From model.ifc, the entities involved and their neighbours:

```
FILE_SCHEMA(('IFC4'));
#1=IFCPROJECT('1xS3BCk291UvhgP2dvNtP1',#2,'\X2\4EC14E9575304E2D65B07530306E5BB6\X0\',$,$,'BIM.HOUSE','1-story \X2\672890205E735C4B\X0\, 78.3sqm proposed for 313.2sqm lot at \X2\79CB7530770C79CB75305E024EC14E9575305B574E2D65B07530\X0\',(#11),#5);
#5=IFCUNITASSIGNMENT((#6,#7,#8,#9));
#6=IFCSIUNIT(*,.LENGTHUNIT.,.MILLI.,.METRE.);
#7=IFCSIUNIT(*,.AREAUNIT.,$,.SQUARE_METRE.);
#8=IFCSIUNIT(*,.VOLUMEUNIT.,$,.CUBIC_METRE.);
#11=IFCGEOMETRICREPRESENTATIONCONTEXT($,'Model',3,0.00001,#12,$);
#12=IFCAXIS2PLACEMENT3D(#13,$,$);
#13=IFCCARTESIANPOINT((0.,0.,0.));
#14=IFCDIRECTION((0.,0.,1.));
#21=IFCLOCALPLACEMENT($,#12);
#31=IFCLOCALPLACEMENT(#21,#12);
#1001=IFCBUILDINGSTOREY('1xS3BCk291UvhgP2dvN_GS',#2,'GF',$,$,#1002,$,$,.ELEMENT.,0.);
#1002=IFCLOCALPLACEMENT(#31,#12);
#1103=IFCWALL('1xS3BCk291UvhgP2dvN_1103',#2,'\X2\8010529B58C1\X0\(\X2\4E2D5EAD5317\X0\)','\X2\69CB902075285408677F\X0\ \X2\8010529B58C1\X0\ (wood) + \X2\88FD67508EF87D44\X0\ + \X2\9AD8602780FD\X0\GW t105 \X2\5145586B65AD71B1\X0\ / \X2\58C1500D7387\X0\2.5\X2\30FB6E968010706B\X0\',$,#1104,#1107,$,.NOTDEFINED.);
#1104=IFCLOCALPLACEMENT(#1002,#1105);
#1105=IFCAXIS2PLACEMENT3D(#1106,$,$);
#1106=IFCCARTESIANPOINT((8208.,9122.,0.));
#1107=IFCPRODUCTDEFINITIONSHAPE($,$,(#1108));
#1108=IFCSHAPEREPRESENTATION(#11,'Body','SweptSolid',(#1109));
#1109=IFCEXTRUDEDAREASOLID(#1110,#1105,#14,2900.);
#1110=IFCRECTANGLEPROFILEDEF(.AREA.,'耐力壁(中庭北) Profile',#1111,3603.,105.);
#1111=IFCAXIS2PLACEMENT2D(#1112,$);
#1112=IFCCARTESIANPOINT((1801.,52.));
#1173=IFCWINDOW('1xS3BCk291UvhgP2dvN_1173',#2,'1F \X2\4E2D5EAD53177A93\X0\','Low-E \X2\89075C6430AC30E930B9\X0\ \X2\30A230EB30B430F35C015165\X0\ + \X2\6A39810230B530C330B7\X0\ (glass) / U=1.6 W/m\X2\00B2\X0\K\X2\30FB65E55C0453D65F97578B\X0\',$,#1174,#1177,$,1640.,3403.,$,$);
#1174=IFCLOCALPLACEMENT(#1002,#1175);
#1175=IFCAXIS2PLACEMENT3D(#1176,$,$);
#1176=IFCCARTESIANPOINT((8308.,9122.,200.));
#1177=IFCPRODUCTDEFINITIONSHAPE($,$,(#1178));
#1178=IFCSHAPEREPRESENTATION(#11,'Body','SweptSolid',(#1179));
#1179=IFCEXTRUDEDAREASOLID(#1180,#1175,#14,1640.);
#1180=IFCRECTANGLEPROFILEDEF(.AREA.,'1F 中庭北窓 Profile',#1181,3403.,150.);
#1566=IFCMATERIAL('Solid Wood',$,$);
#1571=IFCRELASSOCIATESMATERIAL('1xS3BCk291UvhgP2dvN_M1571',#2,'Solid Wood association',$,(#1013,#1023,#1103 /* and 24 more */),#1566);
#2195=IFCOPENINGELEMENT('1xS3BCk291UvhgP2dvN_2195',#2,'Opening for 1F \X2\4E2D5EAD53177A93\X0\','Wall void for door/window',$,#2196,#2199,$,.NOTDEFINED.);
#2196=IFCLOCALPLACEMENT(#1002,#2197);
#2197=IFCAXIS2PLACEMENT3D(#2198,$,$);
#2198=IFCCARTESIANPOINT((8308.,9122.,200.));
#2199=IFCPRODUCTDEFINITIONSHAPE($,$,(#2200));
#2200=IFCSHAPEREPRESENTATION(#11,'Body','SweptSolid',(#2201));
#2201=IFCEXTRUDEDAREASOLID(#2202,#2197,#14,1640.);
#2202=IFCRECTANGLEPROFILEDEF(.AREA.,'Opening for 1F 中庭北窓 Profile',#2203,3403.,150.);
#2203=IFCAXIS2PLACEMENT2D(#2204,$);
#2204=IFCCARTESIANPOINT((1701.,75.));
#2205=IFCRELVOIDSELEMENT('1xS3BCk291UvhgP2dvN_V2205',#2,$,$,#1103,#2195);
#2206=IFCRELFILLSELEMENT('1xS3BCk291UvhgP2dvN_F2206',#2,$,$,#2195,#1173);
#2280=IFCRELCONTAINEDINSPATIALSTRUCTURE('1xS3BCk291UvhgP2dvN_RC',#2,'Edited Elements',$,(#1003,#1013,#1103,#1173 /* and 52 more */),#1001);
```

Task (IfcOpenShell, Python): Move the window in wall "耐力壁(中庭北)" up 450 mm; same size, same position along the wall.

```python
import numpy as np
import ifcopenshell
import ifcopenshell.api.geometry
import ifcopenshell.util.placement
import ifcopenshell.util.unit

model = ifcopenshell.open("model.ifc")
unit_scale = ifcopenshell.util.unit.calculate_unit_scale(model)

window = model.by_guid("1xS3BCk291UvhgP2dvN_1173")
opening = window.FillsVoids[0].RelatingOpeningElement
dz = 450.0

shift = np.array([0.0, 0.0, dz])
# The window is not placed relative to its opening, so move both.
for product in (opening, window):
    matrix = ifcopenshell.util.placement.get_local_placement(product.ObjectPlacement)
    matrix[:3, 3] += shift
    ifcopenshell.api.geometry.edit_object_placement(model, product=product, matrix=matrix, is_si=False)

print(f"moved by {dz * unit_scale:+.3f} m")

model.write("model_rev.ifc")
```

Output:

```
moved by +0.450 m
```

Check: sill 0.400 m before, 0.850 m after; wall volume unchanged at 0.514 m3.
